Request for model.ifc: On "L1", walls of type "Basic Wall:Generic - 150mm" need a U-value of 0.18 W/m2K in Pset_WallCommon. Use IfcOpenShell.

First a look at what the model holds.

```python
import ifcopenshell
import ifcopenshell.util.element

model = ifcopenshell.open("model.ifc")
print(model.schema)
storey = next(s for s in model.by_type("IfcBuildingStorey") if s.Name == "L1")
walls = [e for e in ifcopenshell.util.element.get_decomposition(storey) if e.is_a("IfcWall")]
seen = {}
for e in walls:
    element_type = ifcopenshell.util.element.get_type(e)
    key = (element_type.Name if element_type != e and element_type else None, ifcopenshell.util.element.get_pset(e, "Pset_WallCommon", "ThermalTransmittance"))
    seen[key] = seen.get(key, 0) + 1
for (name, value), count in sorted(seen.items(), key=str):
    print(count, "x", name, "|", value)
```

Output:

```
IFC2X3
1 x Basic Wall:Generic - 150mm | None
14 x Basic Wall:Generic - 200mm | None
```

```python
import ifcopenshell
import ifcopenshell.api.pset
import ifcopenshell.util.element

model = ifcopenshell.open("model.ifc")

storey = next(s for s in model.by_type("IfcBuildingStorey") if s.Name == "L1")
walls = [e for e in ifcopenshell.util.element.get_decomposition(storey) if e.is_a("IfcWall")]

count = 0
for e in walls:
    element_type = ifcopenshell.util.element.get_type(e)
    if element_type in (None, e) or element_type.Name != "Basic Wall:Generic - 150mm":
        continue
    # add_pset returns the element's existing set when there is one.
    pset = ifcopenshell.api.pset.add_pset(model, product=e, name="Pset_WallCommon")
    ifcopenshell.api.pset.edit_pset(model, pset=pset, properties={"ThermalTransmittance": 0.18})
    count += 1

print(count, "walls updated")

model.write("model-out.ifc")
```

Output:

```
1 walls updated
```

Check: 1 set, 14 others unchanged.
